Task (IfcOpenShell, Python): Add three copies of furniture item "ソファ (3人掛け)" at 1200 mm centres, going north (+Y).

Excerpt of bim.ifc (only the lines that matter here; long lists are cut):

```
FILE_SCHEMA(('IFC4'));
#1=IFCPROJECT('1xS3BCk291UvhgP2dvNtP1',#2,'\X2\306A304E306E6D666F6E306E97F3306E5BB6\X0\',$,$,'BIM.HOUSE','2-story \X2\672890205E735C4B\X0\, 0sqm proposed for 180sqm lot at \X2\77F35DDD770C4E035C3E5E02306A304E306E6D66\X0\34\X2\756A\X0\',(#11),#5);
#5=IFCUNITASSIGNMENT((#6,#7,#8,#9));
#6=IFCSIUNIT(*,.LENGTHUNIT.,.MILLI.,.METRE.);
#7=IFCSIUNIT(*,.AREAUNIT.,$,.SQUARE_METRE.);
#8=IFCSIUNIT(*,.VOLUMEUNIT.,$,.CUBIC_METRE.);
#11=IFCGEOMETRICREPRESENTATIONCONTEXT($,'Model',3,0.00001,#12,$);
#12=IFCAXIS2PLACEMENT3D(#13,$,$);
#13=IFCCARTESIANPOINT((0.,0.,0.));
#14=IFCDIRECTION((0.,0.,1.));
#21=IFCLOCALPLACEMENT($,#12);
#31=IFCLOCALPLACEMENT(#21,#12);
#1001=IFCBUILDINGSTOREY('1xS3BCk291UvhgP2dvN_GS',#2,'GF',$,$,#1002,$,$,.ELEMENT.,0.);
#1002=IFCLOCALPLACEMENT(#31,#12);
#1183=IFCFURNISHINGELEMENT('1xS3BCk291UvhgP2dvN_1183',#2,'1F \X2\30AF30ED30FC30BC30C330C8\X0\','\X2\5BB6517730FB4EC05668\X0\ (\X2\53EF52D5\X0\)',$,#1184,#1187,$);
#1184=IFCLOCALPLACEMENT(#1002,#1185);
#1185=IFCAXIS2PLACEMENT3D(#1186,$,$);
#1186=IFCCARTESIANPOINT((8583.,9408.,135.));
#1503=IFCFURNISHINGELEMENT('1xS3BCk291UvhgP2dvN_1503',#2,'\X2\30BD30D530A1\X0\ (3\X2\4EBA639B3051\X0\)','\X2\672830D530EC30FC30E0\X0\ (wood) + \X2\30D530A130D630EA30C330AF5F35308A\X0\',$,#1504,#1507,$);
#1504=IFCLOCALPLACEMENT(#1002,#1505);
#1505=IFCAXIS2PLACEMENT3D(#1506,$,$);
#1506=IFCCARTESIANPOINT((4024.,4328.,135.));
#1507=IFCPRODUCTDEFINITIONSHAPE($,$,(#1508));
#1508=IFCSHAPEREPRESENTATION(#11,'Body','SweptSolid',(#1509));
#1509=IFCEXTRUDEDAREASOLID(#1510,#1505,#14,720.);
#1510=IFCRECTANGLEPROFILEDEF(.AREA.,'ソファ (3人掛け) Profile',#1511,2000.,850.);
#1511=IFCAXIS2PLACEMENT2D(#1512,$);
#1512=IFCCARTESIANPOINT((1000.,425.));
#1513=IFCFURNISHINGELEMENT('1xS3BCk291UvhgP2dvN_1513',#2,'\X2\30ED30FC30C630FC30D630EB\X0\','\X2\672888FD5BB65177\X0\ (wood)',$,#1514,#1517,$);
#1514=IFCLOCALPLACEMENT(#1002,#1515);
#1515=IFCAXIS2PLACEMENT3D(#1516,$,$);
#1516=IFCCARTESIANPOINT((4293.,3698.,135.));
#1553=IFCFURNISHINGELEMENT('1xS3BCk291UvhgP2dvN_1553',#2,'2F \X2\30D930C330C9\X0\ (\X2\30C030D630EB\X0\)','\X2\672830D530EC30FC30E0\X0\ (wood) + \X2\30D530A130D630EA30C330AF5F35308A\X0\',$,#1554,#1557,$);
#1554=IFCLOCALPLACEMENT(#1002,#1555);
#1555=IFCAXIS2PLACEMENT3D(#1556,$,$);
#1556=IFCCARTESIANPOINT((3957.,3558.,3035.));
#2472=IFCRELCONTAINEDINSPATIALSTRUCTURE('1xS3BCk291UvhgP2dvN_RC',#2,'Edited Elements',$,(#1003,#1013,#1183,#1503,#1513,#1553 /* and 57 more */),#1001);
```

```python
import numpy as np
import ifcopenshell
import ifcopenshell.api.geometry
import ifcopenshell.api.root
import ifcopenshell.util.element
import ifcopenshell.util.placement
import ifcopenshell.util.unit

model = ifcopenshell.open("bim.ifc")
unit_scale = ifcopenshell.util.unit.calculate_unit_scale(model)


def reuse_history(source, copy):
    """copy_class also copies each property set's owner history, people and application; keep the originals."""
    for rel in copy.IsDefinedBy:
        if rel.is_a("IfcRelDefinesByProperties") and (history := rel.RelatingPropertyDefinition.OwnerHistory):
            rel.RelatingPropertyDefinition.OwnerHistory = source.OwnerHistory
            ifcopenshell.util.element.remove_deep2(model, history)


source = model.by_guid("1xS3BCk291UvhgP2dvN_1503")
base = ifcopenshell.util.placement.get_local_placement(source.ObjectPlacement)
step = np.array([0.0, 1.0, 0.0]) * 1.2 / unit_scale

for i in range(1, 4):
    copy = ifcopenshell.api.root.copy_class(model, product=source)
    copy.Representation = ifcopenshell.util.element.copy_deep(
        model, source.Representation, exclude=["IfcGeometricRepresentationContext", "IfcRepresentationMap"]
    )
    reuse_history(source, copy)
    matrix = base.copy()
    matrix[:3, 3] += i * step
    print("added at", matrix[:3, 3].round(3) + 0.0)
    ifcopenshell.api.geometry.edit_object_placement(model, product=copy, matrix=matrix, is_si=False)

model.write("bim-out.ifc")
```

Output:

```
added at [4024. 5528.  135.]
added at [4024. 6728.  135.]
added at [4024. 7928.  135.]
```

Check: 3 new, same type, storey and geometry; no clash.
